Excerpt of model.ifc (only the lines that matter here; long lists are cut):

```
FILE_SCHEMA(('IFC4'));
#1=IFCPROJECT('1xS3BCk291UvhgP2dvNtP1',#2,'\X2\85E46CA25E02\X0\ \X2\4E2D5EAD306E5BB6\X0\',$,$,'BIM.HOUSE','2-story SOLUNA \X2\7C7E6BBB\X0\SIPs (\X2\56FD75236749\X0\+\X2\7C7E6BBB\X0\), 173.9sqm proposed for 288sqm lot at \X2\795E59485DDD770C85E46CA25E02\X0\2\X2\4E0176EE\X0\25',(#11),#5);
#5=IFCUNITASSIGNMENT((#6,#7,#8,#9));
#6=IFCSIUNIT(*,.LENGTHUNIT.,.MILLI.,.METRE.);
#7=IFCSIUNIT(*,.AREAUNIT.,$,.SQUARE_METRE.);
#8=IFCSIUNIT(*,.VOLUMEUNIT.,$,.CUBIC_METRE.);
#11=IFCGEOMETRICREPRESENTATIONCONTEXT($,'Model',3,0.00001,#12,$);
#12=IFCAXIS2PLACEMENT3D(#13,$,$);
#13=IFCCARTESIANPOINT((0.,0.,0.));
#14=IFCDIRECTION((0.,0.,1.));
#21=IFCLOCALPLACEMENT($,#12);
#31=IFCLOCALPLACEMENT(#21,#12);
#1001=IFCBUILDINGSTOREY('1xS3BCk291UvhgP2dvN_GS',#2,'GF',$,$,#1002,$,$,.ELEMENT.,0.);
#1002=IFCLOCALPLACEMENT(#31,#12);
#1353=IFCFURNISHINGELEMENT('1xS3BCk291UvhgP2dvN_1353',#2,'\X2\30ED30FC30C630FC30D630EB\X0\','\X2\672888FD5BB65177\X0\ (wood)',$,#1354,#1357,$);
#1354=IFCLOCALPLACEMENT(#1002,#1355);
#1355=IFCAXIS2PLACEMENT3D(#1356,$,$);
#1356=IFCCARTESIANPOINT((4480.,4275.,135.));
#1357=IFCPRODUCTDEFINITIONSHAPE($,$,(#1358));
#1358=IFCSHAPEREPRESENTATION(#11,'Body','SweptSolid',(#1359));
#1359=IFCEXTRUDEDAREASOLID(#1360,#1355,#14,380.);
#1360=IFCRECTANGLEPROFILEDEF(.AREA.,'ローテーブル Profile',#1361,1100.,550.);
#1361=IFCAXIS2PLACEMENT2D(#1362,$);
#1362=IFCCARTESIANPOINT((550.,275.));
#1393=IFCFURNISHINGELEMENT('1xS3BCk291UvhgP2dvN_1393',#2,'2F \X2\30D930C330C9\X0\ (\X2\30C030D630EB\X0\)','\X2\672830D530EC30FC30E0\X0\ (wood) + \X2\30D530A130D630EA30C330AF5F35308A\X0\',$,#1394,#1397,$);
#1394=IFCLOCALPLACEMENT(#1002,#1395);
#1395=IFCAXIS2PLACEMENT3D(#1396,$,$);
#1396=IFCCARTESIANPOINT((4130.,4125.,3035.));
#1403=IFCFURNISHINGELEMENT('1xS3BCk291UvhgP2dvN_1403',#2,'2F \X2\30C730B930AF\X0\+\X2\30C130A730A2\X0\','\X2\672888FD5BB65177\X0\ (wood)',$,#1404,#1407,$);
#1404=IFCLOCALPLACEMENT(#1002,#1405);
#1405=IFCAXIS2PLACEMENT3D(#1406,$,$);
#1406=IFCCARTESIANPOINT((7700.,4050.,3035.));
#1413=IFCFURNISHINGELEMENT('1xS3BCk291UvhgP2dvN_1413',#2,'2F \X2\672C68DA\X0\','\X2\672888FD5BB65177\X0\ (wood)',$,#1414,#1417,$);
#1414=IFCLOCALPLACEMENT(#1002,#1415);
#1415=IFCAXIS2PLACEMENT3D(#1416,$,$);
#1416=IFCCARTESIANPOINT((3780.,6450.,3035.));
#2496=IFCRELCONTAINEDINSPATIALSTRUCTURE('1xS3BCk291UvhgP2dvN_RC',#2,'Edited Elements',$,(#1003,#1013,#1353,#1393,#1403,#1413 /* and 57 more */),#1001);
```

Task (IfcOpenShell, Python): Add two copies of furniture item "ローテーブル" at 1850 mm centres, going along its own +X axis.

```python
import ifcopenshell
import ifcopenshell.api.geometry
import ifcopenshell.api.root
import ifcopenshell.util.element
import ifcopenshell.util.placement

model = ifcopenshell.open("model.ifc")


def reuse_history(source, copy):
    """copy_class also copies each property set's owner history, people and application; keep the originals."""
    for rel in copy.IsDefinedBy:
        if rel.is_a("IfcRelDefinesByProperties") and (history := rel.RelatingPropertyDefinition.OwnerHistory):
            rel.RelatingPropertyDefinition.OwnerHistory = source.OwnerHistory
            ifcopenshell.util.element.remove_deep2(model, history)


source = model.by_guid("1xS3BCk291UvhgP2dvN_1353")
base = ifcopenshell.util.placement.get_local_placement(source.ObjectPlacement)
step = base[:3, 0] * 1850.0

for i in range(1, 3):
    copy = ifcopenshell.api.root.copy_class(model, product=source)
    copy.Representation = ifcopenshell.util.element.copy_deep(
        model, source.Representation, exclude=["IfcGeometricRepresentationContext", "IfcRepresentationMap"]
    )
    reuse_history(source, copy)
    matrix = base.copy()
    matrix[:3, 3] += i * step
    print("added at", matrix[:3, 3].round(3) + 0.0)
    ifcopenshell.api.geometry.edit_object_placement(model, product=copy, matrix=matrix, is_si=False)

model.write("model_v2.ifc")
```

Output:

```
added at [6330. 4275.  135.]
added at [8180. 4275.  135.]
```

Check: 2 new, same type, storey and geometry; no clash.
